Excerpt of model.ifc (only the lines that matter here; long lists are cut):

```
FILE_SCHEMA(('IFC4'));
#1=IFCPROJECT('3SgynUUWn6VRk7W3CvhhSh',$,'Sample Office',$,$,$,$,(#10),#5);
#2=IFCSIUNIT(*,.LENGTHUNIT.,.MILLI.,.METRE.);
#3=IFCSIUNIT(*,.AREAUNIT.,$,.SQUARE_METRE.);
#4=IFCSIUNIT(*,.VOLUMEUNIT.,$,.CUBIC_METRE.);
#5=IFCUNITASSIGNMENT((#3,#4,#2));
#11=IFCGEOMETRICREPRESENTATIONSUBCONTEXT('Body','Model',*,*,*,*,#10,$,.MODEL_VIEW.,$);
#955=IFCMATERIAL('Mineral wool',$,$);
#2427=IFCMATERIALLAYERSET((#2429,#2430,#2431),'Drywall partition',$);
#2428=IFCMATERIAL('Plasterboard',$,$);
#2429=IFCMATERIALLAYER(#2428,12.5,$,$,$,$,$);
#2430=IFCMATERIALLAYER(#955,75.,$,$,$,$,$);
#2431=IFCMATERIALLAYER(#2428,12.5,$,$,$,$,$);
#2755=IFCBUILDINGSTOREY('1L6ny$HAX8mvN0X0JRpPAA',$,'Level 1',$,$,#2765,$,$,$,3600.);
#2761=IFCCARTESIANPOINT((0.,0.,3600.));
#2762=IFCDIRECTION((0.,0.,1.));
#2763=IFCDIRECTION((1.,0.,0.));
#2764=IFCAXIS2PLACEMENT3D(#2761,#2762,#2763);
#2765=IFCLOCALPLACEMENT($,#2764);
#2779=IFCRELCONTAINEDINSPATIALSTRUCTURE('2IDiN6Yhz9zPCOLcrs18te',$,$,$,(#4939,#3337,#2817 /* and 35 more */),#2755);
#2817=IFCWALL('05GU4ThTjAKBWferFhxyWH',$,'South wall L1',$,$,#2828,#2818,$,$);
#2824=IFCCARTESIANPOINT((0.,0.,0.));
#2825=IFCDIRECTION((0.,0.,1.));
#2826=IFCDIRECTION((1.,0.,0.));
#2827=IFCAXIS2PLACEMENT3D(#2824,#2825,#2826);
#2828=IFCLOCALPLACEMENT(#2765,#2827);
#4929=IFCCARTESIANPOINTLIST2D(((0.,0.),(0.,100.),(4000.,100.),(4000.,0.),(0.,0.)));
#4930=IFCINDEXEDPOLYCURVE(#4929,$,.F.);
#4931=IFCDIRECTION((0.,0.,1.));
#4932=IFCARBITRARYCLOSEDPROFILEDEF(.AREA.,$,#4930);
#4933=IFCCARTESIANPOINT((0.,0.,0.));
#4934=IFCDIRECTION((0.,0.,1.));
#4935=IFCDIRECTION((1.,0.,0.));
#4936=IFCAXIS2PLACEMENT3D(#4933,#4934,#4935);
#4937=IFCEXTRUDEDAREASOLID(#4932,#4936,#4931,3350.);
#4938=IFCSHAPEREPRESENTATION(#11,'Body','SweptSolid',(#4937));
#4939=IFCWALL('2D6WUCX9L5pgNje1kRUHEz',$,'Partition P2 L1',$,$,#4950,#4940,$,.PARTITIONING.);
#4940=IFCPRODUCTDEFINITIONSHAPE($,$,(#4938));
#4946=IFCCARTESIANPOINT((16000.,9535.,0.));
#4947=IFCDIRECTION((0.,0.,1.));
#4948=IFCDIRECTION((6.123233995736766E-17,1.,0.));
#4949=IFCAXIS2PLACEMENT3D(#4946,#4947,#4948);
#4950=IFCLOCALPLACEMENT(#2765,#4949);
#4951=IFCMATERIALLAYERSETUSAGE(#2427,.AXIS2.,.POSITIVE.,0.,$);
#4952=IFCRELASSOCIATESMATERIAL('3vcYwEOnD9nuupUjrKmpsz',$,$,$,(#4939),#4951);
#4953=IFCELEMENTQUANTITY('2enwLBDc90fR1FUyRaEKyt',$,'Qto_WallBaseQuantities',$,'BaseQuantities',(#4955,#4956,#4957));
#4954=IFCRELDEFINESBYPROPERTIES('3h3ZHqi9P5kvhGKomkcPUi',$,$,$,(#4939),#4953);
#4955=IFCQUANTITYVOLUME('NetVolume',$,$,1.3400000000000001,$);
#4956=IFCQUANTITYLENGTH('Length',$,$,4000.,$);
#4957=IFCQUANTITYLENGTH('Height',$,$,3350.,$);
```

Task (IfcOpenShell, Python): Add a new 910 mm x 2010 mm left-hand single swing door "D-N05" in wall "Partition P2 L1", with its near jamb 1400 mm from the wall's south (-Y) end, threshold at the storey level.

```python
import numpy as np
import ifcopenshell
import ifcopenshell.api.feature
import ifcopenshell.api.geometry
import ifcopenshell.api.pset
import ifcopenshell.api.root
import ifcopenshell.api.spatial
import ifcopenshell.geom
import ifcopenshell.util.element
import ifcopenshell.util.placement
import ifcopenshell.util.representation
import ifcopenshell.util.shape
import ifcopenshell.util.unit

model = ifcopenshell.open("model.ifc")
unit_scale = ifcopenshell.util.unit.calculate_unit_scale(model)
volume_scale = ifcopenshell.util.unit.calculate_unit_scale(model, "VOLUMEUNIT")
settings = ifcopenshell.geom.settings()


def volume(element):
    """Net volume in cubic metres, openings subtracted."""
    shape = ifcopenshell.geom.create_shape(settings, element)
    return ifcopenshell.util.shape.get_volume(shape.geometry)


wall = model.by_guid("2D6WUCX9L5pgNje1kRUHEz")
storey = ifcopenshell.util.element.get_container(wall, ifc_class="IfcBuildingStorey")
context = ifcopenshell.util.representation.get_context(model, "Model", "Body", "MODEL_VIEW")
before = volume(wall)

width, height, from_end, sill = 0.91, 2.01, 1.4, 0.0  # metres

# The wall runs along its own X axis, and the end named is its -X end.
wall_shape = ifcopenshell.geom.create_shape(settings, wall)
x, y, z = ifcopenshell.util.shape.get_vertices(wall_shape.geometry).T
start = x.min() + from_end
face, thickness = float(y.min()), float(y.max() - y.min())
wall_matrix = ifcopenshell.util.placement.get_local_placement(wall.ObjectPlacement)
level = ifcopenshell.util.placement.get_local_placement(storey.ObjectPlacement)[2, 3]


def in_wall(x, y):
    """Placement at x, y metres in the wall's axes, at sill height."""
    matrix = wall_matrix.copy()
    matrix[:, 3] = wall_matrix @ np.array([x / unit_scale, y / unit_scale, 0.0, 1.0])
    matrix[2, 3] = level + sill / unit_scale
    return matrix


# Opening: a box that overshoots both wall faces by 50 mm.
opening = ifcopenshell.api.root.create_entity(model, ifc_class="IfcOpeningElement", predefined_type="OPENING")
box = ifcopenshell.api.geometry.add_wall_representation(
    model, context=context, length=width, height=height, thickness=thickness + 0.1
)
ifcopenshell.api.geometry.assign_representation(model, product=opening, representation=box)
ifcopenshell.api.geometry.edit_object_placement(model, product=opening, matrix=in_wall(start, face - 0.05), is_si=False)
ifcopenshell.api.feature.add_feature(model, feature=opening, element=wall)

door = ifcopenshell.api.root.create_entity(model, ifc_class="IfcDoor", name="D-N05", predefined_type="DOOR")
door.OverallWidth, door.OverallHeight = width / unit_scale, height / unit_scale
door.OperationType = "SINGLE_SWING_LEFT"
body = ifcopenshell.api.geometry.add_door_representation(
    model,
    context=context,
    overall_width=door.OverallWidth,
    overall_height=door.OverallHeight,
    operation_type="SINGLE_SWING_LEFT",
    lining_properties={"LiningDepth": thickness / unit_scale, "ThresholdDepth": thickness / unit_scale},
)
ifcopenshell.api.geometry.assign_representation(model, product=door, representation=body)
ifcopenshell.api.spatial.assign_container(model, products=[door], relating_structure=storey)
ifcopenshell.api.feature.add_filling(model, opening=opening, element=door)

# The lining spans the wall, so the door starts at the wall face.
ifcopenshell.api.geometry.edit_object_placement(model, product=door, matrix=in_wall(start, face), is_si=False)

after = volume(wall)

# Update the wall's stored quantities.
qto = model.by_id(ifcopenshell.util.element.get_pset(wall, "Qto_WallBaseQuantities", should_inherit=False)["id"])
ifcopenshell.api.pset.edit_qto(model, qto=qto, properties={"NetVolume": after / volume_scale})

print(f"wall volume {before:.3f} -> {after:.3f} m3")

model.write("model_v2.ifc")
```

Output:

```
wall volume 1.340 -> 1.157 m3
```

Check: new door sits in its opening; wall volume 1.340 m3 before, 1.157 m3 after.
